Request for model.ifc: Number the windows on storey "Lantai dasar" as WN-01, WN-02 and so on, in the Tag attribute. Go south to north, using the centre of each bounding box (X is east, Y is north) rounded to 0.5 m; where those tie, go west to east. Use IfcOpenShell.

First a look at what the model holds.

```python
import ifcopenshell
import ifcopenshell.util.element
import ifcopenshell.util.placement

model = ifcopenshell.open("model.ifc")
print(model.schema)
storey = next(s for s in model.by_type("IfcBuildingStorey") if s.Name == "Lantai dasar")
windows = [e for e in ifcopenshell.util.element.get_decomposition(storey) if e.is_a("IfcWindow")]
for e in sorted(windows, key=lambda e: e.id()):
    origin = ifcopenshell.util.placement.get_local_placement(e.ObjectPlacement)[:3, 3]
    print(e.id(), e.Tag, e.Name, origin.round(2) + 0.0, sep=" | ")
```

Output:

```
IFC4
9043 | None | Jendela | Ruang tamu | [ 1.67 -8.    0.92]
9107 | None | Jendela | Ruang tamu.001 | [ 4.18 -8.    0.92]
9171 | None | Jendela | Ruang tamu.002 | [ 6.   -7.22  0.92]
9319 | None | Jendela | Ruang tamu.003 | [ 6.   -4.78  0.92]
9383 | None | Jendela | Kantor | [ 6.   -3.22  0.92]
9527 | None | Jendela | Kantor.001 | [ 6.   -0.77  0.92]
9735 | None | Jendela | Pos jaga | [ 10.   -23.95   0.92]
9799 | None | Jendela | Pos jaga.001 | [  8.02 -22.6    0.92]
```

```python
import ifcopenshell
import ifcopenshell.geom
import ifcopenshell.util.element
import ifcopenshell.util.shape

model = ifcopenshell.open("model.ifc")
settings = ifcopenshell.geom.settings()
settings.set("use-world-coords", True)


def centre(element):
    shape = ifcopenshell.geom.create_shape(settings, element)
    return ifcopenshell.util.shape.get_bbox_centroid(shape.geometry)


storey = next(s for s in model.by_type("IfcBuildingStorey") if s.Name == "Lantai dasar")
windows = [e for e in ifcopenshell.util.element.get_decomposition(storey) if e.is_a("IfcWindow")]

# Insertion points can sit at a corner or the storey origin, so sort by the geometry (in metres).
centres = {e: centre(e) for e in windows}
windows.sort(key=lambda e: (round(centres[e][1] / 0.5), centres[e][0]))

for i, e in enumerate(windows, start=1):
    number = f"WN-{i:02d}"
    e.Tag = number
    print(e.id(), number)

model.write("model_rev.ifc")
```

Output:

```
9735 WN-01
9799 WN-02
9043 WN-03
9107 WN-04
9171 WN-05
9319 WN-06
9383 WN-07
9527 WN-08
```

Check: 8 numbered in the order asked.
